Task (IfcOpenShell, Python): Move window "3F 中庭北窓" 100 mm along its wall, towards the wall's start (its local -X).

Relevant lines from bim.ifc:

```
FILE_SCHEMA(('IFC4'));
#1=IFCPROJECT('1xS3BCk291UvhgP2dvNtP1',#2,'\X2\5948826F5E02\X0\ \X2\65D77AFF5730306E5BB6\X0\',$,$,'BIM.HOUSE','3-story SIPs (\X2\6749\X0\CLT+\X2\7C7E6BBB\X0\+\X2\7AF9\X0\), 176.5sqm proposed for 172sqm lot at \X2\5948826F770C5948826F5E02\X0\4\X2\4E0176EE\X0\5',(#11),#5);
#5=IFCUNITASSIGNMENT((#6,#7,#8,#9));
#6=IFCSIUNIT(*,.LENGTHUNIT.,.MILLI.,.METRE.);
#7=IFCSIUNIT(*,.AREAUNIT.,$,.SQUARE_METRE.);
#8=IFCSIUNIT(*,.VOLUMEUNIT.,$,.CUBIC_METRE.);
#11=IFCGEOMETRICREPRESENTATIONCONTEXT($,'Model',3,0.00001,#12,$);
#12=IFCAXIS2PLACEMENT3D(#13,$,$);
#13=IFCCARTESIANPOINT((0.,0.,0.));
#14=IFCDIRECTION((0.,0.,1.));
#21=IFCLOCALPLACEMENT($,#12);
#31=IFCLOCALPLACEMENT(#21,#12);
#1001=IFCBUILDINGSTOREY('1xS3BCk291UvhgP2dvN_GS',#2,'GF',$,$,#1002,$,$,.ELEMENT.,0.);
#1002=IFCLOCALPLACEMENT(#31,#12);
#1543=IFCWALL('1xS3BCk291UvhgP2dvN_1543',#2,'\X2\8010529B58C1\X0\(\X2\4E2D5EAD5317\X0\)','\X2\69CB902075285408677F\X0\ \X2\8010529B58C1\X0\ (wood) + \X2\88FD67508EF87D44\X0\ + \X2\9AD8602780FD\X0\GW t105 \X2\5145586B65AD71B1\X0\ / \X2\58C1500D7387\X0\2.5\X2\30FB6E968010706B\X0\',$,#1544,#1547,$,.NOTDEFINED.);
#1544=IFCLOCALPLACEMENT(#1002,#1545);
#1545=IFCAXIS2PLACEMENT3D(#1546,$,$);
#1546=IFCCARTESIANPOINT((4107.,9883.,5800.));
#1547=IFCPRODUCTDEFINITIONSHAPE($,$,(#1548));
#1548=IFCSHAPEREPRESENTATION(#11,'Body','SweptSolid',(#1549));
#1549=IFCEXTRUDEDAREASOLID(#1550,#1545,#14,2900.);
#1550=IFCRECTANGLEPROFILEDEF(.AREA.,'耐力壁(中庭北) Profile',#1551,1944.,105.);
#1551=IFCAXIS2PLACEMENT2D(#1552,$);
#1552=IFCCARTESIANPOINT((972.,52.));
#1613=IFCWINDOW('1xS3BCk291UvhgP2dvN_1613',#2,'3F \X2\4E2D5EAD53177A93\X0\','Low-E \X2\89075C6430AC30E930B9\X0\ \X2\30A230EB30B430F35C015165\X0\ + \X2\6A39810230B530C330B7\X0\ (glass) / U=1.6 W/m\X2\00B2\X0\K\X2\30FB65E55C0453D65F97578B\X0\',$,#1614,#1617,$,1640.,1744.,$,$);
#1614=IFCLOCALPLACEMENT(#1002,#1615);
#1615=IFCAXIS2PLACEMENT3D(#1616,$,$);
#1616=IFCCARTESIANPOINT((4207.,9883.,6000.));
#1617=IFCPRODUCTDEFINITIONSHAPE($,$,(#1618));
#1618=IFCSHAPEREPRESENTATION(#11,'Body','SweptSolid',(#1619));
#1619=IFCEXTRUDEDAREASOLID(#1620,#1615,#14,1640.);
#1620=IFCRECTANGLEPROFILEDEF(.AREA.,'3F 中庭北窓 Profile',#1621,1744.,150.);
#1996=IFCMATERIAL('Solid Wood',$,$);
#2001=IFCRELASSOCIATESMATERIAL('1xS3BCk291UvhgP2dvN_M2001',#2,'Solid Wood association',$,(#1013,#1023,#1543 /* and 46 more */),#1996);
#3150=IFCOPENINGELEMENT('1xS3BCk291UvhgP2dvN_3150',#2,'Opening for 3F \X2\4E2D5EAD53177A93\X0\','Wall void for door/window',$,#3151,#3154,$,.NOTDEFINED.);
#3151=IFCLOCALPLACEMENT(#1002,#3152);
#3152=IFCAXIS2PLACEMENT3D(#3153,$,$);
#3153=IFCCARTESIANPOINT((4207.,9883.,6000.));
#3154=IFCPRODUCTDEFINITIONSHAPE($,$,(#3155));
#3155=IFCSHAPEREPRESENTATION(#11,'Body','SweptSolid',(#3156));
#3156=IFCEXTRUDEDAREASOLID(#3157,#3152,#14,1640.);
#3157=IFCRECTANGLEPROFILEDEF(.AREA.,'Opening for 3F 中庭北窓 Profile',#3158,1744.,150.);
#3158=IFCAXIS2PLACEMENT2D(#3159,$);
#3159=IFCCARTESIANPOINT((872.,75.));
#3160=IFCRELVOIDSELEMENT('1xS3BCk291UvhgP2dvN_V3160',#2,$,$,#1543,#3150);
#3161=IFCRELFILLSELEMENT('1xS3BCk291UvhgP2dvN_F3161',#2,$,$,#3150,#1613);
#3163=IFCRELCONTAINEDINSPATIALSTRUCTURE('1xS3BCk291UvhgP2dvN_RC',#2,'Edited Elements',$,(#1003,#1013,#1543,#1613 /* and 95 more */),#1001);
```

```python
import ifcopenshell
import ifcopenshell.api.geometry
import ifcopenshell.util.placement

model = ifcopenshell.open("bim.ifc")

window = model.by_id(1613)
opening = window.FillsVoids[0].RelatingOpeningElement
wall = opening.VoidsElements[0].RelatingBuildingElement

wall_matrix = ifcopenshell.util.placement.get_local_placement(wall.ObjectPlacement)
shift = wall_matrix[:3, 0] * -100.0
before = ifcopenshell.util.placement.get_local_placement(window.ObjectPlacement)[:3, 3].copy()

# The window is not placed relative to its opening, so move both.
for product in (opening, window):
    matrix = ifcopenshell.util.placement.get_local_placement(product.ObjectPlacement)
    matrix[:3, 3] += shift
    ifcopenshell.api.geometry.edit_object_placement(model, product=product, matrix=matrix, is_si=False)

after = ifcopenshell.util.placement.get_local_placement(window.ObjectPlacement)[:3, 3]
print("window moved by", (after - before).round(3) + 0.0)

model.write("bim_v2.ifc")
```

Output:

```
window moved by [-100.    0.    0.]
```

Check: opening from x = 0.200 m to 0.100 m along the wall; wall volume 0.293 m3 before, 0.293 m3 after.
